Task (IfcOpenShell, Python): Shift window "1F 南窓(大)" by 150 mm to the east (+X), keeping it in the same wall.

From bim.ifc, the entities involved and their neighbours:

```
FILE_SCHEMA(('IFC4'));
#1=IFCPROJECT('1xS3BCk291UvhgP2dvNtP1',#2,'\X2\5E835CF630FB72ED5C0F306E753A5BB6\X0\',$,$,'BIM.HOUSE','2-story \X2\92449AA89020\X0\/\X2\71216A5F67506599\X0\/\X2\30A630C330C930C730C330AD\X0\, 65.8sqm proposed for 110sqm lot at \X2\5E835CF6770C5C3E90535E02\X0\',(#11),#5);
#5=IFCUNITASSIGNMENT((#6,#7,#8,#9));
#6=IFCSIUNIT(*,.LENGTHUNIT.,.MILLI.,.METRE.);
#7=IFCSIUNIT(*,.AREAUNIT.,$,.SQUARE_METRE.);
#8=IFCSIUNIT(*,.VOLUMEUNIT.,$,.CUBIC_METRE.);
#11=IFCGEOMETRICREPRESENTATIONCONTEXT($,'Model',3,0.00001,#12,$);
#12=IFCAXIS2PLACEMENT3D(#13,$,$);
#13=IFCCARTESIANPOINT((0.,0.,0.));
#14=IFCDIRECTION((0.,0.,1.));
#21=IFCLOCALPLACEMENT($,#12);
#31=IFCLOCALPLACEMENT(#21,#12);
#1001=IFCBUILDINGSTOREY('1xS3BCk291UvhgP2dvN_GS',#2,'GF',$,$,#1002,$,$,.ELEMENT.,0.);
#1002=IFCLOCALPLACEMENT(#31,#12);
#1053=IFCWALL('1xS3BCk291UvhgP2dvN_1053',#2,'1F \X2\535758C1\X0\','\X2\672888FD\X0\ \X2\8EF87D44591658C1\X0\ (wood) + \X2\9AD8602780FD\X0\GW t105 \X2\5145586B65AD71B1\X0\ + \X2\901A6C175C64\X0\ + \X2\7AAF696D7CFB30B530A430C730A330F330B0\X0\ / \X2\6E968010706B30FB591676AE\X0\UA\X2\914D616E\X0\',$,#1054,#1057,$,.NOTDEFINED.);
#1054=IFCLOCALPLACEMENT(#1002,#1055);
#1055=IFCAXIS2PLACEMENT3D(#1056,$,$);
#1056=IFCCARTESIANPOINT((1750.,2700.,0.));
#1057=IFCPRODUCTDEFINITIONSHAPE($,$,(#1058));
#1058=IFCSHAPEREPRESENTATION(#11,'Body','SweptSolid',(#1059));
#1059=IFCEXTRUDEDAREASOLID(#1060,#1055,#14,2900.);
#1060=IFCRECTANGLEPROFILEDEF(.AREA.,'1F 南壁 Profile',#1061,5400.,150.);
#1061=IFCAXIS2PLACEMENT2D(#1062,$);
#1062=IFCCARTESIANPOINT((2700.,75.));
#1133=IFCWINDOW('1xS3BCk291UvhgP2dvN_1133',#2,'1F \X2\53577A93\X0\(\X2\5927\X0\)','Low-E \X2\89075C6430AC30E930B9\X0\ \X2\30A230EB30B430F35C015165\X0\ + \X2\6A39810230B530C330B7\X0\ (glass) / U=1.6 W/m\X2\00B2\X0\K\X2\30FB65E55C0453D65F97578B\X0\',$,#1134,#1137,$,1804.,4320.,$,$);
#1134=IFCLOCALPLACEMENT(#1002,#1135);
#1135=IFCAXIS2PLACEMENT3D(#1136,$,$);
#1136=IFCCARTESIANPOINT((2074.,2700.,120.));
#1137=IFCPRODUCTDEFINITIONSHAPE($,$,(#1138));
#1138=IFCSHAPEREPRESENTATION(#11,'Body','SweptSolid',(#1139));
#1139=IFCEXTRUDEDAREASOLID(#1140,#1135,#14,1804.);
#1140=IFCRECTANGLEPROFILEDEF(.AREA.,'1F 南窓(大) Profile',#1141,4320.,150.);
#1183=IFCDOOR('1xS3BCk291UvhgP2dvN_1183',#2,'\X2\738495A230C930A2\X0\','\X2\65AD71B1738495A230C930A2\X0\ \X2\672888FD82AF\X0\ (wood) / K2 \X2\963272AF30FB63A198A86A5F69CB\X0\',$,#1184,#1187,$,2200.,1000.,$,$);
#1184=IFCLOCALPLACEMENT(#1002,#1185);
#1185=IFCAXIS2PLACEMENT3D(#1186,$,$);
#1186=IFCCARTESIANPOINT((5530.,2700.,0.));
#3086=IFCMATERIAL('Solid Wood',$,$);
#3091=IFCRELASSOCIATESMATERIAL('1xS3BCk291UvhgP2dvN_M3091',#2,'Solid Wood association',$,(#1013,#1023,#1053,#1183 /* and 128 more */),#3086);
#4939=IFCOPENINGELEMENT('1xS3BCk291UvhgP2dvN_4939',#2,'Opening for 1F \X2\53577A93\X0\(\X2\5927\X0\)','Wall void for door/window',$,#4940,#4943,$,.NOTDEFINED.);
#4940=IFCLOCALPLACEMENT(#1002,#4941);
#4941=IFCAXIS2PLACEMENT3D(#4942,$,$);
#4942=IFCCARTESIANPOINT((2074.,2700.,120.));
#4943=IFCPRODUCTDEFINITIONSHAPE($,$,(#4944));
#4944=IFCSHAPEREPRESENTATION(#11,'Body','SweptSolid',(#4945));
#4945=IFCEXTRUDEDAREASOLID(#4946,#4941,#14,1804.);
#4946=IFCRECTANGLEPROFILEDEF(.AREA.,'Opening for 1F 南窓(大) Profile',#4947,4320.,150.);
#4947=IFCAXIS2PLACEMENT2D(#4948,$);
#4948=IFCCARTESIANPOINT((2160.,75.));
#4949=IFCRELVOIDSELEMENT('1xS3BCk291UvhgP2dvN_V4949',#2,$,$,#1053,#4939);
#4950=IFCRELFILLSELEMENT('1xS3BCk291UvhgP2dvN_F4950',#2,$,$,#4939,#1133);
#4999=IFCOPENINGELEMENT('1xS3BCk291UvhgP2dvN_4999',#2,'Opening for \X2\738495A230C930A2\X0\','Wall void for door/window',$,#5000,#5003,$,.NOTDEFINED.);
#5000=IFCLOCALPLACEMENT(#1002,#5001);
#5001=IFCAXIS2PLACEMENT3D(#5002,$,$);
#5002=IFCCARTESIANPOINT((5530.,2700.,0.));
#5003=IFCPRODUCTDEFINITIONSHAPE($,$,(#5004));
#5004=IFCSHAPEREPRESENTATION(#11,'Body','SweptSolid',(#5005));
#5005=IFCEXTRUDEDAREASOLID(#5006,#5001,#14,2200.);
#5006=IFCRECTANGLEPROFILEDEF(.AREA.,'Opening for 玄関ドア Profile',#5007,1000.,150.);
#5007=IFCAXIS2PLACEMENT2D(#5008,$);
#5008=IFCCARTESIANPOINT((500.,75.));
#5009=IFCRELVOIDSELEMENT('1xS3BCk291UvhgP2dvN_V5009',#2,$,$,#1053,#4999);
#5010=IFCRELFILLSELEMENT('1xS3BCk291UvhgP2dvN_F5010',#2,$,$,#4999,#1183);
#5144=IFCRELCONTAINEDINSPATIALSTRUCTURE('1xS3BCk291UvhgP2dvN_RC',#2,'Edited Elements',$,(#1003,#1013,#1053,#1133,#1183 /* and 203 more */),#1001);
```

```python
import ifcopenshell
import ifcopenshell.api.geometry
import ifcopenshell.util.placement
import ifcopenshell.util.unit

model = ifcopenshell.open("bim.ifc")
unit_scale = ifcopenshell.util.unit.calculate_unit_scale(model)

window = model.by_id(1133)
opening = window.FillsVoids[0].RelatingOpeningElement
wall = opening.VoidsElements[0].RelatingBuildingElement

wall_matrix = ifcopenshell.util.placement.get_local_placement(wall.ObjectPlacement)
shift = wall_matrix[:3, 0] * 0.15 / unit_scale
before = ifcopenshell.util.placement.get_local_placement(window.ObjectPlacement)[:3, 3].copy()

# The window is not placed relative to its opening, so move both.
for product in (opening, window):
    matrix = ifcopenshell.util.placement.get_local_placement(product.ObjectPlacement)
    matrix[:3, 3] += shift
    ifcopenshell.api.geometry.edit_object_placement(model, product=product, matrix=matrix, is_si=False)

after = ifcopenshell.util.placement.get_local_placement(window.ObjectPlacement)[:3, 3]
print("window moved by", (after - before).round(3) + 0.0)

model.write("bim-out.ifc")
```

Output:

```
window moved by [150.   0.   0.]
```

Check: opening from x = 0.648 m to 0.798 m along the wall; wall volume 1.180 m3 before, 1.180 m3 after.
